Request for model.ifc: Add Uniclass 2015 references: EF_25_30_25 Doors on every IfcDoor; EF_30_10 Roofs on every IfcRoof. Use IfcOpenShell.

First a look at what the model holds.

```python
import ifcopenshell

model = ifcopenshell.open("model.ifc")
print(model.schema)
print("classifications:", [c.Name for c in model.by_type("IfcClassification")])
for ifc_class in ("IfcDoor", "IfcRoof", "IfcStair", "IfcWall", "IfcWindow"):
    print(ifc_class, len(model.by_type(ifc_class)))
```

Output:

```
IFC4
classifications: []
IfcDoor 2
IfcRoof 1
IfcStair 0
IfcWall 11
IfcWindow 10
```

```python
import ifcopenshell
import ifcopenshell.api.classification

model = ifcopenshell.open("model.ifc")

system = ifcopenshell.api.classification.add_classification(model, classification="Uniclass 2015")

codes = {
    "IfcDoor": ("EF_25_30_25", "Doors"),
    "IfcRoof": ("EF_30_10", "Roofs"),
}
for ifc_class, (code, name) in codes.items():
    products = model.by_type(ifc_class)
    ifcopenshell.api.classification.add_reference(
        model, products=products, classification=system, identification=code, name=name
    )
    print(code, len(products))

model.write("model_edited.ifc")
```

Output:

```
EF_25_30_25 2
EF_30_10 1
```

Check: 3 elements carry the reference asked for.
